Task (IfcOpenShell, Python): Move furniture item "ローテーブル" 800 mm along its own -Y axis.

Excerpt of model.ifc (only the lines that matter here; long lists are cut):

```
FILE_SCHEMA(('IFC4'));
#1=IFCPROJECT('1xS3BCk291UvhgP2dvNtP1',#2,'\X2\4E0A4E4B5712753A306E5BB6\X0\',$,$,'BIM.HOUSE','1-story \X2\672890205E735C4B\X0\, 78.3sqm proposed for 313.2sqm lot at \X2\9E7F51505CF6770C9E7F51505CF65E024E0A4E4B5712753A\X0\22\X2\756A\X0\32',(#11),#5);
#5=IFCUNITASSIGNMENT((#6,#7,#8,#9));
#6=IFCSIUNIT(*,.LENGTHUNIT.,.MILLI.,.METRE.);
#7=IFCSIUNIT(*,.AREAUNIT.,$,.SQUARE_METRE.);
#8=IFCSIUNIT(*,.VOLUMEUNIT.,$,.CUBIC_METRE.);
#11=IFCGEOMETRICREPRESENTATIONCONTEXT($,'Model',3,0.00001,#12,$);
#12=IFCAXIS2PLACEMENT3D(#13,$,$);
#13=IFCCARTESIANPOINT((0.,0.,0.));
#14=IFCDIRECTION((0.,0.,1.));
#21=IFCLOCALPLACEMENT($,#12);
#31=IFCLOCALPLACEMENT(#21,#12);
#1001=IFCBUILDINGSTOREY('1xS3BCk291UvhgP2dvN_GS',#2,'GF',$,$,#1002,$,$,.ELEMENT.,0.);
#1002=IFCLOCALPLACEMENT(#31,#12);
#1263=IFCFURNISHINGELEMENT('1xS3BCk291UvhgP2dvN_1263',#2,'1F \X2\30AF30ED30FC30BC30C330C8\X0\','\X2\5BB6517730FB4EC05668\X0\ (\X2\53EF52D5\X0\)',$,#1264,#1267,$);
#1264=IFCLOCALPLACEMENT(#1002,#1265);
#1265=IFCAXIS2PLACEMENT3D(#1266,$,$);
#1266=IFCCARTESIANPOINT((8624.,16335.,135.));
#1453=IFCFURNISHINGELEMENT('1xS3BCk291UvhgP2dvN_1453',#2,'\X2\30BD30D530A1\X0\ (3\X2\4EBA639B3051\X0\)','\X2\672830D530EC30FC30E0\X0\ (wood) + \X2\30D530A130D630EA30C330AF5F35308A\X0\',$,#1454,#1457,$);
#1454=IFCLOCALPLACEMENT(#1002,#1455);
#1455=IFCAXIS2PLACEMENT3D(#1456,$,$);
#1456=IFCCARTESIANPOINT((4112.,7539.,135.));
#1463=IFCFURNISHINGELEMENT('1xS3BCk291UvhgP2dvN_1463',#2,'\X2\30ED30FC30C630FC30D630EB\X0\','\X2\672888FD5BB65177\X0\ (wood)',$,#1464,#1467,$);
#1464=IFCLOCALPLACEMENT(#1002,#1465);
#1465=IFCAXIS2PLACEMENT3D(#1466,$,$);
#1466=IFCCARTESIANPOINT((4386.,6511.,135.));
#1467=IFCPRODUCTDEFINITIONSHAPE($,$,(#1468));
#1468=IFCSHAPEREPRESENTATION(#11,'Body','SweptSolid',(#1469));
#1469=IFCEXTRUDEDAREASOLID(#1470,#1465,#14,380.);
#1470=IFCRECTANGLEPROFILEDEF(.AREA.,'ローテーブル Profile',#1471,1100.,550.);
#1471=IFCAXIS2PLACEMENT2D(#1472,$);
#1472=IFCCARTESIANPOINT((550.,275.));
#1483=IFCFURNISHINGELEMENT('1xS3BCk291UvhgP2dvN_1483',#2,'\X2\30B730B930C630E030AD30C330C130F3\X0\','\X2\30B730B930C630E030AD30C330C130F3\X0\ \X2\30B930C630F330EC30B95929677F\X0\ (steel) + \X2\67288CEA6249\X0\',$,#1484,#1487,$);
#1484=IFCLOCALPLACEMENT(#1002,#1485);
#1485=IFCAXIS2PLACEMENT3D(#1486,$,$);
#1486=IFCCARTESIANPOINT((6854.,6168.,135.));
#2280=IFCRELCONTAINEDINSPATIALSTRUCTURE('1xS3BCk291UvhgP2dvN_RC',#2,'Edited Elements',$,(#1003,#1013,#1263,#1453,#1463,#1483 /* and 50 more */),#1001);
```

```python
import ifcopenshell
import ifcopenshell.api.geometry
import ifcopenshell.util.placement

model = ifcopenshell.open("model.ifc")

item = model.by_guid("1xS3BCk291UvhgP2dvN_1463")
matrix = ifcopenshell.util.placement.get_local_placement(item.ObjectPlacement)
matrix[:3, 3] -= matrix[:3, 1] * 800.0
ifcopenshell.api.geometry.edit_object_placement(model, product=item, matrix=matrix, is_si=False)

print(ifcopenshell.util.placement.get_local_placement(item.ObjectPlacement).round(3) + 0.0)

model.write("model_updated.ifc")
```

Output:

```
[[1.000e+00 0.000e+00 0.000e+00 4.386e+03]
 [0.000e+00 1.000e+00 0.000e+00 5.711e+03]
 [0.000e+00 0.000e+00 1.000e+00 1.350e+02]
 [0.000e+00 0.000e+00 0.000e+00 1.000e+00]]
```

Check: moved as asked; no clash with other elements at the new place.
